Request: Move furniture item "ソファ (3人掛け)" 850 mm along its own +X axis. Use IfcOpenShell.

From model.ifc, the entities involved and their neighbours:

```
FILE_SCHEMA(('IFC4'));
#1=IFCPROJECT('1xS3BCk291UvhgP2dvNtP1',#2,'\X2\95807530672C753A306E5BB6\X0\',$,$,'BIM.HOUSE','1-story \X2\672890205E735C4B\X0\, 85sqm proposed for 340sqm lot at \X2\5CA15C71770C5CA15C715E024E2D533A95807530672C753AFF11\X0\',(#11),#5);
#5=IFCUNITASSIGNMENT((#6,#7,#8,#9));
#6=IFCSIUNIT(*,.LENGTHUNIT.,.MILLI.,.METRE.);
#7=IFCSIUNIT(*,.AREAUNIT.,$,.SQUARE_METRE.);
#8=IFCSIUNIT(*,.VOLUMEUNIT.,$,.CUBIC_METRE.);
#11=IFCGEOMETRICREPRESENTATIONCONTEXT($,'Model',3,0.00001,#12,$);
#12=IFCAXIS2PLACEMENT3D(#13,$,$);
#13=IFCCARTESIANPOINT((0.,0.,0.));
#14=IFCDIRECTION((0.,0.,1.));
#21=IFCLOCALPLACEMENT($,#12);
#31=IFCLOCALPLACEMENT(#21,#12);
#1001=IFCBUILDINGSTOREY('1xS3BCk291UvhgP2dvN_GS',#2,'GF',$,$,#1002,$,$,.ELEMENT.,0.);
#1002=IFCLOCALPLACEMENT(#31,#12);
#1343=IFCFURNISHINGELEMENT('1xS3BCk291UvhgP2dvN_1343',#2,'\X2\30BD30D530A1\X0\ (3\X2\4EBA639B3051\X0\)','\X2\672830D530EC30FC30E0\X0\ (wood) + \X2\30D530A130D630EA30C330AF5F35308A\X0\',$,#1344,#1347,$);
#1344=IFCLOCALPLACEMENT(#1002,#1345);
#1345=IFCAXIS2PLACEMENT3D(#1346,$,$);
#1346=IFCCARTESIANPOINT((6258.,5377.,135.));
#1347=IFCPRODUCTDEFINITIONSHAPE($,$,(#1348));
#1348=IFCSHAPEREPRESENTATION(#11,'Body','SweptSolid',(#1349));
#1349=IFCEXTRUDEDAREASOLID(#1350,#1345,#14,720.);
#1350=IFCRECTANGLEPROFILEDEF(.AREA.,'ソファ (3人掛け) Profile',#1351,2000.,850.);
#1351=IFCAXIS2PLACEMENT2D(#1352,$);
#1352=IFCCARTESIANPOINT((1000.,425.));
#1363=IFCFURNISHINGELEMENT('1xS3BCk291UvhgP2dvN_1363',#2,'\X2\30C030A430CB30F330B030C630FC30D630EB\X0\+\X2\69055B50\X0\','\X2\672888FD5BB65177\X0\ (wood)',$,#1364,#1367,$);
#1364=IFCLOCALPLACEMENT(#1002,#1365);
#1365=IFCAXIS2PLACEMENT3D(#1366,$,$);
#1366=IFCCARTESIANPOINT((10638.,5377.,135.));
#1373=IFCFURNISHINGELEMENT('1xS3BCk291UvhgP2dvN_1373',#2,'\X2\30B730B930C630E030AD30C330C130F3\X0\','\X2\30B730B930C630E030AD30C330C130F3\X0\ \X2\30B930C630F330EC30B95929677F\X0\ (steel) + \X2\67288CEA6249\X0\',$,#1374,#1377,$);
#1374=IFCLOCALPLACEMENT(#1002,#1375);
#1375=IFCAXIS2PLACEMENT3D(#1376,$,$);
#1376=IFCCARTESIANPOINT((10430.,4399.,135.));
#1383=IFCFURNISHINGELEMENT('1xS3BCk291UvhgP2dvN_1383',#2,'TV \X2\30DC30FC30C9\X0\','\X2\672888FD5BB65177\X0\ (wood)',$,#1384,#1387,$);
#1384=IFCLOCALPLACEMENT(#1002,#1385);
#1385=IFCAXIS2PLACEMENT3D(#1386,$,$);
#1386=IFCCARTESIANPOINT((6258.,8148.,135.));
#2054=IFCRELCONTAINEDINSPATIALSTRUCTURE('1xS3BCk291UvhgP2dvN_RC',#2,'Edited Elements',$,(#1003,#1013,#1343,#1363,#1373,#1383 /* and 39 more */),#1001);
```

```python
import ifcopenshell
import ifcopenshell.api.geometry
import ifcopenshell.util.placement

model = ifcopenshell.open("model.ifc")

item = model.by_guid("1xS3BCk291UvhgP2dvN_1343")
matrix = ifcopenshell.util.placement.get_local_placement(item.ObjectPlacement)
matrix[:3, 3] += matrix[:3, 0] * 850.0
ifcopenshell.api.geometry.edit_object_placement(model, product=item, matrix=matrix, is_si=False)

print(ifcopenshell.util.placement.get_local_placement(item.ObjectPlacement).round(3) + 0.0)

model.write("model_v2.ifc")
```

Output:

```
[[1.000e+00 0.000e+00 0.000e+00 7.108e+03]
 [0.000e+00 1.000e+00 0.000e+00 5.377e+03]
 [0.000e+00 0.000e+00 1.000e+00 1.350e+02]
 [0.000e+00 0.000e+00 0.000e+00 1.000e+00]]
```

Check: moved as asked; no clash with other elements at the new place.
